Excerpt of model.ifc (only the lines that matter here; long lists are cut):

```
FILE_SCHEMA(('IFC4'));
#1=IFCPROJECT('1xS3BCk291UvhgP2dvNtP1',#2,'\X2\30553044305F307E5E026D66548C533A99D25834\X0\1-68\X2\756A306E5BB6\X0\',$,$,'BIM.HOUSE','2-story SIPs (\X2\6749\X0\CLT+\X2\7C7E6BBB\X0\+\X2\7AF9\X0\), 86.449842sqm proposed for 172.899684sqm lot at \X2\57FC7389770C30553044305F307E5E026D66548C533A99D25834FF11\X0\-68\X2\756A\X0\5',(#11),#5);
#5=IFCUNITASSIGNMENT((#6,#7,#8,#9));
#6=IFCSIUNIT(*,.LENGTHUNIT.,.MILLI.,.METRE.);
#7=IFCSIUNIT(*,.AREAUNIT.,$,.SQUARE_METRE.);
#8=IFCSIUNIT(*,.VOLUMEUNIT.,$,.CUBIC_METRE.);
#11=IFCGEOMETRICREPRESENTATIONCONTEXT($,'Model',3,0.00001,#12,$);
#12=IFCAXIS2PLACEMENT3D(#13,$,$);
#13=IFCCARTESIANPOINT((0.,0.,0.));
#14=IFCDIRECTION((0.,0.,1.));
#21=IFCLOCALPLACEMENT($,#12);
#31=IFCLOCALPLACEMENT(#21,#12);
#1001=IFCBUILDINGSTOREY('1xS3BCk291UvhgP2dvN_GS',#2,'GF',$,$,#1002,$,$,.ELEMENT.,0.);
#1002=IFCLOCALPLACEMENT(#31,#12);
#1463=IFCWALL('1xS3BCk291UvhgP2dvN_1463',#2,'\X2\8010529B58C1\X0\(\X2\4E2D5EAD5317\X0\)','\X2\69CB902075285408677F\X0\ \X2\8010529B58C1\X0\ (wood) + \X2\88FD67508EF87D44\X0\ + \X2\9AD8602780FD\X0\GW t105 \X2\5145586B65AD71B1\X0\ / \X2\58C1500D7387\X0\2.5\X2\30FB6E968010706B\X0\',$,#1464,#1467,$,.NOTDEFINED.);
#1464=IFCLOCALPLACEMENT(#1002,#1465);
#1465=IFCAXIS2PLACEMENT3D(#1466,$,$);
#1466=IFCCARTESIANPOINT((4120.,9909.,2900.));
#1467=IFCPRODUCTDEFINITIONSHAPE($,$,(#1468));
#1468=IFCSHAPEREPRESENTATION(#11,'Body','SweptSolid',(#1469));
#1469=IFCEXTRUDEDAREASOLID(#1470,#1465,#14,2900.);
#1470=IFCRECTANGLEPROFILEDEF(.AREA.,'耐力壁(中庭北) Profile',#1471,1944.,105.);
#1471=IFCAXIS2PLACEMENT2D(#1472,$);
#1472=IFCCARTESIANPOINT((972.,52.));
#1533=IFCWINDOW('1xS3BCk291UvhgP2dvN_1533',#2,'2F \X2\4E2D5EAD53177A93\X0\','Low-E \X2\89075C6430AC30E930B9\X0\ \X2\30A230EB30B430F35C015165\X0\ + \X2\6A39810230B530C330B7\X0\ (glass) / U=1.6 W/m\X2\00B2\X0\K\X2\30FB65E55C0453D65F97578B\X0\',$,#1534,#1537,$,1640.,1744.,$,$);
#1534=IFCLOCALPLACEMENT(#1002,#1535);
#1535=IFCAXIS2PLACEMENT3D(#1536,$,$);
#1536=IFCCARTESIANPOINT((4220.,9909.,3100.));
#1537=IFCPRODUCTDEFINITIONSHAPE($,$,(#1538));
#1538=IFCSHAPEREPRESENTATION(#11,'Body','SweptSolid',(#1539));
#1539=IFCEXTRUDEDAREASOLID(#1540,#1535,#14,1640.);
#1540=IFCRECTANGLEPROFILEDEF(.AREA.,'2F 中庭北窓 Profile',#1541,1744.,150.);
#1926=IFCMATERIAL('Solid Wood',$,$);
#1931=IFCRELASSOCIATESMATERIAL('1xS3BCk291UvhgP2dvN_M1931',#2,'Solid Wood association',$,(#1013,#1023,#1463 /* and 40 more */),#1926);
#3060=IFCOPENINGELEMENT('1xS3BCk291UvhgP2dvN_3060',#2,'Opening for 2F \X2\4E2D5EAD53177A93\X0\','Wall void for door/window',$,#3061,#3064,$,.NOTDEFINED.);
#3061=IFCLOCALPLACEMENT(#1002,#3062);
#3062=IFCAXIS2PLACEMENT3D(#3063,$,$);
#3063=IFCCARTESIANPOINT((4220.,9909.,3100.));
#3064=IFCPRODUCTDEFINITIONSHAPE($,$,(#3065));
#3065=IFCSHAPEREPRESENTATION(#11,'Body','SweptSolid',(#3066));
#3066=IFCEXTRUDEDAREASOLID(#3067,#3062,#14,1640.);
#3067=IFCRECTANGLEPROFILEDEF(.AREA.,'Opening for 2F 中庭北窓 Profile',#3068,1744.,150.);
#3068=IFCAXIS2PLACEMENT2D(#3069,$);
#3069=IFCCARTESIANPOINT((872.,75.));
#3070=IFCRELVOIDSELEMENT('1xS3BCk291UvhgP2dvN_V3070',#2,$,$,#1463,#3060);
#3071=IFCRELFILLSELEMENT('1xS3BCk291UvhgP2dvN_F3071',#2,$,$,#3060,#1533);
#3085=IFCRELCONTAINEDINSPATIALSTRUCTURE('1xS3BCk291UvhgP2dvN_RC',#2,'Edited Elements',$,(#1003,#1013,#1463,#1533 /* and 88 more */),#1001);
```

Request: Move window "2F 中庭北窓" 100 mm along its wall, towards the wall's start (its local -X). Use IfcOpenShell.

```python
import ifcopenshell
import ifcopenshell.api.geometry
import ifcopenshell.util.placement

model = ifcopenshell.open("model.ifc")

window = model.by_guid("1xS3BCk291UvhgP2dvN_1533")
opening = window.FillsVoids[0].RelatingOpeningElement
wall = opening.VoidsElements[0].RelatingBuildingElement

wall_matrix = ifcopenshell.util.placement.get_local_placement(wall.ObjectPlacement)
shift = wall_matrix[:3, 0] * -100.0
before = ifcopenshell.util.placement.get_local_placement(window.ObjectPlacement)[:3, 3].copy()

# The window is not placed relative to its opening, so move both.
for product in (opening, window):
    matrix = ifcopenshell.util.placement.get_local_placement(product.ObjectPlacement)
    matrix[:3, 3] += shift
    ifcopenshell.api.geometry.edit_object_placement(model, product=product, matrix=matrix, is_si=False)

after = ifcopenshell.util.placement.get_local_placement(window.ObjectPlacement)[:3, 3]
print("window moved by", (after - before).round(3) + 0.0)

model.write("model-out.ifc")
```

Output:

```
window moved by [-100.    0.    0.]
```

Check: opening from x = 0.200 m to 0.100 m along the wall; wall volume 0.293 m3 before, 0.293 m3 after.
